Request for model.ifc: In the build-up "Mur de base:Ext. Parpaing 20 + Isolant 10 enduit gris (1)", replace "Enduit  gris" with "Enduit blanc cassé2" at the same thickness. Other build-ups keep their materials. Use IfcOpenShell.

First a look at what the model holds.

```python
import ifcopenshell
import ifcopenshell.util.element

model = ifcopenshell.open("model.ifc")
print(model.schema)
for layer_set in model.by_type("IfcMaterialLayerSet"):
    if layer_set.LayerSetName == "Mur de base:Ext. Parpaing 20 + Isolant 10 enduit gris (1)":
        for layer in layer_set.MaterialLayers:
            print(layer.id(), layer.Material and layer.Material.Name, layer.LayerThickness, sep=" | ")
        print(len(ifcopenshell.util.element.get_elements_by_material(model, layer_set)), "elements and types use it")
print(sorted(m.Name for m in model.by_type("IfcMaterial") if m.Name)[:60])
```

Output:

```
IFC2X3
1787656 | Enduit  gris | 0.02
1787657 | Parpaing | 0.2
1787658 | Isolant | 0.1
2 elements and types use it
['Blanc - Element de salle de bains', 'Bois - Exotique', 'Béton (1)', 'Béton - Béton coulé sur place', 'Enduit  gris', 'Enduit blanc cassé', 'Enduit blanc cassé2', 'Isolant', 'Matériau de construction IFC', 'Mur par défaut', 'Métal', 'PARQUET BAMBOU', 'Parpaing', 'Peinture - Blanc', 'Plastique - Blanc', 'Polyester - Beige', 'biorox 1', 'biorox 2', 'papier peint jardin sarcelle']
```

```python
import ifcopenshell
import ifcopenshell.api.material

model = ifcopenshell.open("model.ifc")

layer_set = next(s for s in model.by_type("IfcMaterialLayerSet") if s.LayerSetName == "Mur de base:Ext. Parpaing 20 + Isolant 10 enduit gris (1)")
layer = next(l for l in layer_set.MaterialLayers if l.Material and l.Material.Name == "Enduit  gris")
material = next(m for m in model.by_type("IfcMaterial") if m.Name == "Enduit blanc cassé2")

# Point this one layer at the other material; renaming the old one would change it everywhere.
ifcopenshell.api.material.edit_layer(model, layer=layer, attributes={}, material=material)

print([l.Material.Name if l.Material else None for l in layer_set.MaterialLayers])

model.write("model_v2.ifc")
```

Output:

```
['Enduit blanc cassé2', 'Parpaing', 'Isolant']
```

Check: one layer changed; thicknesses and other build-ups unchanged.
